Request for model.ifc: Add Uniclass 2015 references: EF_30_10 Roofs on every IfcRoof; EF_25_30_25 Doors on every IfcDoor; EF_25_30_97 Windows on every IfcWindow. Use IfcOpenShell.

First a look at what the model holds.

```python
import ifcopenshell

model = ifcopenshell.open("model.ifc")
print(model.schema)
print("classifications:", [c.Name for c in model.by_type("IfcClassification")])
for ifc_class in ("IfcDoor", "IfcRoof", "IfcStair", "IfcWall", "IfcWindow"):
    print(ifc_class, len(model.by_type(ifc_class)))
```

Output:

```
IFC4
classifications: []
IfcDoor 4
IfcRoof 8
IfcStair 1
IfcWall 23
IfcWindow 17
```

```python
import ifcopenshell
import ifcopenshell.api.classification

model = ifcopenshell.open("model.ifc")

system = ifcopenshell.api.classification.add_classification(model, classification="Uniclass 2015")

codes = {
    "IfcRoof": ("EF_30_10", "Roofs"),
    "IfcDoor": ("EF_25_30_25", "Doors"),
    "IfcWindow": ("EF_25_30_97", "Windows"),
}
for ifc_class, (code, name) in codes.items():
    products = model.by_type(ifc_class)
    ifcopenshell.api.classification.add_reference(
        model, products=products, classification=system, identification=code, name=name
    )
    print(code, len(products))

model.write("model_rev.ifc")
```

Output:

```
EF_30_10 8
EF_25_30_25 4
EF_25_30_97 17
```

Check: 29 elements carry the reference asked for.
